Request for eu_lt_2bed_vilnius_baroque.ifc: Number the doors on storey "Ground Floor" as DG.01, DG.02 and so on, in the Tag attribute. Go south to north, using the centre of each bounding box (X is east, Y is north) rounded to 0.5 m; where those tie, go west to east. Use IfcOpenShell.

First a look at what the model holds.

```python
import ifcopenshell
import ifcopenshell.util.element
import ifcopenshell.util.placement

model = ifcopenshell.open("eu_lt_2bed_vilnius_baroque.ifc")
print(model.schema)
storey = next(s for s in model.by_type("IfcBuildingStorey") if s.Name == "Ground Floor")
doors = [e for e in ifcopenshell.util.element.get_decomposition(storey) if e.is_a("IfcDoor")]
for e in sorted(doors, key=lambda e: e.id()):
    origin = ifcopenshell.util.placement.get_local_placement(e.ObjectPlacement)[:3, 3]
    print(e.id(), e.Tag, e.Name, origin.round(2) + 0.0, sep=" | ")
```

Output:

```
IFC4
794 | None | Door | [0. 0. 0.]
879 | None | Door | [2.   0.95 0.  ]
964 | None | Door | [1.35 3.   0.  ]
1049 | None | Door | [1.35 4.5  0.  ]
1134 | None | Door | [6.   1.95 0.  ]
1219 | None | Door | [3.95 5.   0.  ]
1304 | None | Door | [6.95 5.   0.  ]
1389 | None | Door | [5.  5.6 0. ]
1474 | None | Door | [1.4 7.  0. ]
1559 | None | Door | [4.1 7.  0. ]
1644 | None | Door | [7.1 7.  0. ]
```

```python
import ifcopenshell
import ifcopenshell.geom
import ifcopenshell.util.element
import ifcopenshell.util.shape

model = ifcopenshell.open("eu_lt_2bed_vilnius_baroque.ifc")
settings = ifcopenshell.geom.settings()
settings.set("use-world-coords", True)


def centre(element):
    shape = ifcopenshell.geom.create_shape(settings, element)
    return ifcopenshell.util.shape.get_bbox_centroid(shape.geometry)


storey = next(s for s in model.by_type("IfcBuildingStorey") if s.Name == "Ground Floor")
doors = [e for e in ifcopenshell.util.element.get_decomposition(storey) if e.is_a("IfcDoor")]

# Insertion points can sit at a corner or the storey origin, so sort by the geometry (in metres).
centres = {e: centre(e) for e in doors}
doors.sort(key=lambda e: (round(centres[e][1] / 0.5), centres[e][0]))

for i, e in enumerate(doors, start=1):
    number = f"DG.{i:02d}"
    e.Tag = number
    print(e.id(), number)

model.write("eu_lt_2bed_vilnius_baroque_edited.ifc")
```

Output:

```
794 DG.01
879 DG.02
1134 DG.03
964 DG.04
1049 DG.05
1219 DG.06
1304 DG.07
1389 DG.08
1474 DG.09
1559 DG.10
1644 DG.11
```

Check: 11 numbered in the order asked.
